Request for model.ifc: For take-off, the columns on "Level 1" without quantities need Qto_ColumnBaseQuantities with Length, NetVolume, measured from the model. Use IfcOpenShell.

First a look at what the model holds.

```python
import ifcopenshell
import ifcopenshell.util.element
import ifcopenshell.util.unit

model = ifcopenshell.open("model.ifc")
print(model.schema)
for unit_type in ("LENGTHUNIT", "AREAUNIT", "VOLUMEUNIT"):
    print(unit_type, ifcopenshell.util.unit.calculate_unit_scale(model, unit_type))
storey = next(s for s in model.by_type("IfcBuildingStorey") if s.Name == "Level 1")
columns = [e for e in ifcopenshell.util.element.get_decomposition(storey) if e.is_a("IfcColumn")]
for e in sorted(columns, key=lambda e: e.id()):
    print(e.id(), e.is_a(), e.Name, list(ifcopenshell.util.element.get_psets(e, qtos_only=True)), sep=" | ")
```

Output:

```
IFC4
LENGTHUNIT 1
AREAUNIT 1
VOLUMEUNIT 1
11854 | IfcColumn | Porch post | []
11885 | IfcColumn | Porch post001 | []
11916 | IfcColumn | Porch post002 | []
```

```python
import ifcopenshell
import ifcopenshell.api.pset
import ifcopenshell.geom
import ifcopenshell.util.element
import ifcopenshell.util.shape
import ifcopenshell.util.unit

model = ifcopenshell.open("model.ifc")
unit_scale = ifcopenshell.util.unit.calculate_unit_scale(model)
volume_scale = ifcopenshell.util.unit.calculate_unit_scale(model, "VOLUMEUNIT")
settings = ifcopenshell.geom.settings()

storey = next(s for s in model.by_type("IfcBuildingStorey") if s.Name == "Level 1")
columns = [e for e in ifcopenshell.util.element.get_decomposition(storey) if e.is_a("IfcColumn")]

for e in sorted(columns, key=lambda e: e.id()):
    if ifcopenshell.util.element.get_psets(e, qtos_only=True, should_inherit=False):
        continue
    # Geometry comes back in metres, in the element's own axes.
    shape = ifcopenshell.geom.create_shape(settings, e)
    values = {
        "Length": ifcopenshell.util.shape.get_z(shape.geometry) / unit_scale,
        "NetVolume": ifcopenshell.util.shape.get_volume(shape.geometry) / volume_scale,
    }
    qto = ifcopenshell.api.pset.add_qto(model, product=e, name="Qto_ColumnBaseQuantities")
    ifcopenshell.api.pset.edit_qto(model, qto=qto, properties=values)
    print(e.id(), {k: round(v, 3) for k, v in values.items()})

model.write("model_updated.ifc")
```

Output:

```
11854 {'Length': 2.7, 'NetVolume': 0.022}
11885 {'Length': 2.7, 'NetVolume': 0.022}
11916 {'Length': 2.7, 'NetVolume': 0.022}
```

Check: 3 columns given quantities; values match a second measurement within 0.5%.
